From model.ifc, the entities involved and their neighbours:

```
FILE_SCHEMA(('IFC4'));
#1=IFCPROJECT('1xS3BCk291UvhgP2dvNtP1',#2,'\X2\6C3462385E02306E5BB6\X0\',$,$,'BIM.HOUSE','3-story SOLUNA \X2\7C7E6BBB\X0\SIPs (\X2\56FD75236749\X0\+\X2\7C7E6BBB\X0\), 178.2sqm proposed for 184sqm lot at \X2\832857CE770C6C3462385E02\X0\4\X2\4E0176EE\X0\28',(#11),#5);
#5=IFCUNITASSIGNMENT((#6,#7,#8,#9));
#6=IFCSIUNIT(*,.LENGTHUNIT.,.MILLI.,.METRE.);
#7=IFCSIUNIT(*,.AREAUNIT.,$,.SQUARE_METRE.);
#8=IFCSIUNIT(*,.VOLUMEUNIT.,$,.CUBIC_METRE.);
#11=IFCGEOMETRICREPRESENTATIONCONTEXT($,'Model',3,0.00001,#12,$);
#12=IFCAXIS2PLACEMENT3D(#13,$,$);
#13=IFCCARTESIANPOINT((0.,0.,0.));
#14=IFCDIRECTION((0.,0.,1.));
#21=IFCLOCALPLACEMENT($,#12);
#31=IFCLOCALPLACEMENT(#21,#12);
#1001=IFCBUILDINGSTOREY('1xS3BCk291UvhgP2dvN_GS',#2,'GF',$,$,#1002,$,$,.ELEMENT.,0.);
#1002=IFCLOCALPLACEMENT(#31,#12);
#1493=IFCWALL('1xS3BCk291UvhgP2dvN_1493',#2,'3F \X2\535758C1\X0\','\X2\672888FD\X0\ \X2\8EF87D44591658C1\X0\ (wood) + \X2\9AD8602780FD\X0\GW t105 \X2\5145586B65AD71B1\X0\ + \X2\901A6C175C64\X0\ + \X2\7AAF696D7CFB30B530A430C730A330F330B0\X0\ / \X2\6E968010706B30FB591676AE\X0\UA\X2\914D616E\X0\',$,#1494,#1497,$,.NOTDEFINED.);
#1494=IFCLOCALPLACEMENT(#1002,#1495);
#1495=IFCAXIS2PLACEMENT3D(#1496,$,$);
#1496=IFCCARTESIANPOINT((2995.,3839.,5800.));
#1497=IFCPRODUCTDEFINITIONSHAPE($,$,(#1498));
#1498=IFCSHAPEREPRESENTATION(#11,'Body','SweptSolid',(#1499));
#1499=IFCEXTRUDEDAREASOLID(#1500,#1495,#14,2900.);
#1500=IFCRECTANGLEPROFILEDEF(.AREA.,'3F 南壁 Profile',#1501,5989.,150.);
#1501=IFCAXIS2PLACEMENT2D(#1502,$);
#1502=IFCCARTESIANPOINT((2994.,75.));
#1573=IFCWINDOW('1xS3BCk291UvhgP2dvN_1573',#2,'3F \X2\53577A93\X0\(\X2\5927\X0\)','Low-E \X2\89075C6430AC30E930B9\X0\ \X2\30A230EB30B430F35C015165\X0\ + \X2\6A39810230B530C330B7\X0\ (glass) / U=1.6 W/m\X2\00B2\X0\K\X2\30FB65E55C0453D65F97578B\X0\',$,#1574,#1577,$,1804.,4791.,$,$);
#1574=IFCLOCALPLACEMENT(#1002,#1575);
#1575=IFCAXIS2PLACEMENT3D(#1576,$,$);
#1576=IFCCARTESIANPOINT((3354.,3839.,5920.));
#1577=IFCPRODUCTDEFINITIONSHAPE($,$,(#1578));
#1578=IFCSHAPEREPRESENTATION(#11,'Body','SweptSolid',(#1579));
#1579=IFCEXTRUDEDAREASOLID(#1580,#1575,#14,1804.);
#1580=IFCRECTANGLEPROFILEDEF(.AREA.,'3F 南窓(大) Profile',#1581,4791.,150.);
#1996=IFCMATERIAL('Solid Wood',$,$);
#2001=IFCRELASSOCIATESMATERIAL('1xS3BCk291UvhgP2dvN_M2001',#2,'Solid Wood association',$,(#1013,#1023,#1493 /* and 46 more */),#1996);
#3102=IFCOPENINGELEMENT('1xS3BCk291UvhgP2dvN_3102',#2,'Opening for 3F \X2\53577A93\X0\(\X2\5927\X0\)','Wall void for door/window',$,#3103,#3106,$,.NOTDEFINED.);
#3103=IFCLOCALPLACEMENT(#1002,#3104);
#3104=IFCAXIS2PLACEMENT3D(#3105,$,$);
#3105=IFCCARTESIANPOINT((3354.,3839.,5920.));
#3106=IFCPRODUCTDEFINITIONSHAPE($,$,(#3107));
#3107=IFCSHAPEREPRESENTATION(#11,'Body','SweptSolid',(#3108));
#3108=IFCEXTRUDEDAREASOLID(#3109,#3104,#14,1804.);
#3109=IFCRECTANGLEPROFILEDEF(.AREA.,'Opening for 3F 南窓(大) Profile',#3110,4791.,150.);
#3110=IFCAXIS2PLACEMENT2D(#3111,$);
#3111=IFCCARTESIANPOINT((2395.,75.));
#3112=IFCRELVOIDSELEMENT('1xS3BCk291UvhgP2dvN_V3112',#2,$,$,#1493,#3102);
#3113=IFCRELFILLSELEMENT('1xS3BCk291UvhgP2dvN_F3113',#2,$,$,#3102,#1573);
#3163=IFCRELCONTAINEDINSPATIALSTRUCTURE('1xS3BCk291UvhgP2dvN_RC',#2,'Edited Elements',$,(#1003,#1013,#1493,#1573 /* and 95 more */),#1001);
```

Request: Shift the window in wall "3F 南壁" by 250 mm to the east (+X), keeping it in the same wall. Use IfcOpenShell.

```python
import ifcopenshell
import ifcopenshell.api.geometry
import ifcopenshell.util.placement

model = ifcopenshell.open("model.ifc")

window = model.by_id(1573)
opening = window.FillsVoids[0].RelatingOpeningElement
wall = opening.VoidsElements[0].RelatingBuildingElement

wall_matrix = ifcopenshell.util.placement.get_local_placement(wall.ObjectPlacement)
shift = wall_matrix[:3, 0] * 250.0
before = ifcopenshell.util.placement.get_local_placement(window.ObjectPlacement)[:3, 3].copy()

# The window is not placed relative to its opening, so move both.
for product in (opening, window):
    matrix = ifcopenshell.util.placement.get_local_placement(product.ObjectPlacement)
    matrix[:3, 3] += shift
    ifcopenshell.api.geometry.edit_object_placement(model, product=product, matrix=matrix, is_si=False)

after = ifcopenshell.util.placement.get_local_placement(window.ObjectPlacement)[:3, 3]
print("window moved by", (after - before).round(3) + 0.0)

model.write("model-out.ifc")
```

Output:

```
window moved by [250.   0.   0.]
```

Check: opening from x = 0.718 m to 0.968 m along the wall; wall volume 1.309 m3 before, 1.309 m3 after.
